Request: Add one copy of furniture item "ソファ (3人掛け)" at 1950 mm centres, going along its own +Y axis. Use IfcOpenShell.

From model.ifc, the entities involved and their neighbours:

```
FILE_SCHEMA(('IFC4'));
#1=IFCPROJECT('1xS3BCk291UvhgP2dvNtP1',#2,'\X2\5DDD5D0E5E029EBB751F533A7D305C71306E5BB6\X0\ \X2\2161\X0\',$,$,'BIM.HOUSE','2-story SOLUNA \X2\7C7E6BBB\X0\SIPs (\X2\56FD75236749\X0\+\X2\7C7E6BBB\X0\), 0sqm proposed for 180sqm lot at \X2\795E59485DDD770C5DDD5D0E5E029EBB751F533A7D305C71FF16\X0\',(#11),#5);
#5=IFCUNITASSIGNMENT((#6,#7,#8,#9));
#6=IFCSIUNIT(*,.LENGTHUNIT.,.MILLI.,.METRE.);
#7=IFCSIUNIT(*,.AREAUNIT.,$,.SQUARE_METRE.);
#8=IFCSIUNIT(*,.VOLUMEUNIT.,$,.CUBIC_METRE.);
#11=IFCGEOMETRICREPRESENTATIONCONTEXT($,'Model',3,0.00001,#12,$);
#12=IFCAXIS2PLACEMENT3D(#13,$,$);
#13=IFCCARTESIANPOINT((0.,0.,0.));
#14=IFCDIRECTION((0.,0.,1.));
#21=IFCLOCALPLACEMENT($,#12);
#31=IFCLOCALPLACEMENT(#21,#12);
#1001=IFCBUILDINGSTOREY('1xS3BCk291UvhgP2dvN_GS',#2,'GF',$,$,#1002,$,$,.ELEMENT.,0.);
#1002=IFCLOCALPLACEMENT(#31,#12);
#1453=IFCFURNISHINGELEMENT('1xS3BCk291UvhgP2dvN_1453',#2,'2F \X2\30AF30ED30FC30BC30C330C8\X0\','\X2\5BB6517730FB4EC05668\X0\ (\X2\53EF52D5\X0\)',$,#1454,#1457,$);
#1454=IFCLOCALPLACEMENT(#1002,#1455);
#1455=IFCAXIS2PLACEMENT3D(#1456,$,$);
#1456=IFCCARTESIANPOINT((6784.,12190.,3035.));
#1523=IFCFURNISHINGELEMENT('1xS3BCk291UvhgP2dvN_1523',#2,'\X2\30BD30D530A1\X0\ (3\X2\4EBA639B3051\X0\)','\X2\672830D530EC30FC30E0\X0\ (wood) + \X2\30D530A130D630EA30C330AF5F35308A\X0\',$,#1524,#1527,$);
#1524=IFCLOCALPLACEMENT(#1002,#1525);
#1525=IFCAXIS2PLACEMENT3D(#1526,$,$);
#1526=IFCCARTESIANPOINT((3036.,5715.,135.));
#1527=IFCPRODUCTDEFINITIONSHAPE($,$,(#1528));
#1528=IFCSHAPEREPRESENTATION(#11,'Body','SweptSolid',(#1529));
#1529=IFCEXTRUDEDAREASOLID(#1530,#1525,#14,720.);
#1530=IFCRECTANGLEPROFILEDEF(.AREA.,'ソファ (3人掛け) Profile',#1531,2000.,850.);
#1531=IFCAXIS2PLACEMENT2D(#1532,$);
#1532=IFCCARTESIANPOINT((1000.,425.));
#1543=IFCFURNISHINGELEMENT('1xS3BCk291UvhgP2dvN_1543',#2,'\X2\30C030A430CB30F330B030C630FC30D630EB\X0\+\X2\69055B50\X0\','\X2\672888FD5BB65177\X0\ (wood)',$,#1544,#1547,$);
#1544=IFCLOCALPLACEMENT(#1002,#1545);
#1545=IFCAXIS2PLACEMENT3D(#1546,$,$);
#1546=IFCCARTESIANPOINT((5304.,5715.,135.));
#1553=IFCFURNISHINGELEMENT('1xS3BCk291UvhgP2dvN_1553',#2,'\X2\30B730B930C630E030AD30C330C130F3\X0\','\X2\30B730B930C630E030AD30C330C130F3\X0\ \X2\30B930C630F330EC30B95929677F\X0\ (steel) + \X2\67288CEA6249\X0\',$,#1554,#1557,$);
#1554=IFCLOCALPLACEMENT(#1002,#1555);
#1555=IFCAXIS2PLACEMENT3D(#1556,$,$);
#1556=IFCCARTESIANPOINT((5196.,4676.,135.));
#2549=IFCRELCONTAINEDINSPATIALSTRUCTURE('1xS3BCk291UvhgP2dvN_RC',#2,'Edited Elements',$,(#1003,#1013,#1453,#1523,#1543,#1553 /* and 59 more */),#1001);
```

```python
import ifcopenshell
import ifcopenshell.api.geometry
import ifcopenshell.api.root
import ifcopenshell.util.element
import ifcopenshell.util.placement
import ifcopenshell.util.unit

model = ifcopenshell.open("model.ifc")
unit_scale = ifcopenshell.util.unit.calculate_unit_scale(model)


def reuse_history(source, copy):
    """copy_class also copies each property set's owner history, people and application; keep the originals."""
    for rel in copy.IsDefinedBy:
        if rel.is_a("IfcRelDefinesByProperties") and (history := rel.RelatingPropertyDefinition.OwnerHistory):
            rel.RelatingPropertyDefinition.OwnerHistory = source.OwnerHistory
            ifcopenshell.util.element.remove_deep2(model, history)


source = model.by_guid("1xS3BCk291UvhgP2dvN_1523")
base = ifcopenshell.util.placement.get_local_placement(source.ObjectPlacement)
step = base[:3, 1] * 1.95 / unit_scale

for i in range(1, 2):
    copy = ifcopenshell.api.root.copy_class(model, product=source)
    copy.Representation = ifcopenshell.util.element.copy_deep(
        model, source.Representation, exclude=["IfcGeometricRepresentationContext", "IfcRepresentationMap"]
    )
    reuse_history(source, copy)
    matrix = base.copy()
    matrix[:3, 3] += i * step
    print("added at", matrix[:3, 3].round(3) + 0.0)
    ifcopenshell.api.geometry.edit_object_placement(model, product=copy, matrix=matrix, is_si=False)

model.write("model_edited.ifc")
```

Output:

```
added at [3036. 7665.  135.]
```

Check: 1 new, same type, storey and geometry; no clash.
